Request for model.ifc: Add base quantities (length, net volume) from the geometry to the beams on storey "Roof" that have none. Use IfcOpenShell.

First a look at what the model holds.

```python
import ifcopenshell
import ifcopenshell.util.element
import ifcopenshell.util.unit

model = ifcopenshell.open("model.ifc")
print(model.schema)
for unit_type in ("LENGTHUNIT", "AREAUNIT", "VOLUMEUNIT"):
    print(unit_type, ifcopenshell.util.unit.calculate_unit_scale(model, unit_type))
storey = next(s for s in model.by_type("IfcBuildingStorey") if s.Name == "Roof")
beams = [e for e in ifcopenshell.util.element.get_decomposition(storey) if e.is_a("IfcBeam")]
for e in sorted(beams, key=lambda e: e.id()):
    print(e.id(), e.is_a(), e.Name, list(ifcopenshell.util.element.get_psets(e, qtos_only=True)), sep=" | ")
```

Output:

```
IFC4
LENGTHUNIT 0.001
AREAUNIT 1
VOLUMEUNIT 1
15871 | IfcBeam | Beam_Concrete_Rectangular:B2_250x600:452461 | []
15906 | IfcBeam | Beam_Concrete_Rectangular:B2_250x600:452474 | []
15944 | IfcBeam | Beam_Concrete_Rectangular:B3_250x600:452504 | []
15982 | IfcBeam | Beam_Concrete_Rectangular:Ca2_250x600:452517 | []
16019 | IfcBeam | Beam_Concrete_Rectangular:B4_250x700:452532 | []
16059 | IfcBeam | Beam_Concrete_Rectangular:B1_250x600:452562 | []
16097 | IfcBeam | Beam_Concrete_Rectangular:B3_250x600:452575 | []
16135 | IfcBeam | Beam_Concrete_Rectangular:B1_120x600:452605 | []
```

```python
import ifcopenshell
import ifcopenshell.api.pset
import ifcopenshell.geom
import ifcopenshell.util.element
import ifcopenshell.util.shape
import ifcopenshell.util.unit

model = ifcopenshell.open("model.ifc")
unit_scale = ifcopenshell.util.unit.calculate_unit_scale(model)
volume_scale = ifcopenshell.util.unit.calculate_unit_scale(model, "VOLUMEUNIT")
settings = ifcopenshell.geom.settings()

storey = next(s for s in model.by_type("IfcBuildingStorey") if s.Name == "Roof")
beams = [e for e in ifcopenshell.util.element.get_decomposition(storey) if e.is_a("IfcBeam")]

for e in sorted(beams, key=lambda e: e.id()):
    if ifcopenshell.util.element.get_psets(e, qtos_only=True, should_inherit=False):
        continue
    # Geometry comes back in metres, in the element's own axes.
    shape = ifcopenshell.geom.create_shape(settings, e)
    values = {
        "Length": ifcopenshell.util.shape.get_max_xyz(shape.geometry) / unit_scale,
        "NetVolume": ifcopenshell.util.shape.get_volume(shape.geometry) / volume_scale,
    }
    qto = ifcopenshell.api.pset.add_qto(model, product=e, name="Qto_BeamBaseQuantities")
    ifcopenshell.api.pset.edit_qto(model, qto=qto, properties=values)
    print(e.id(), {k: round(v, 3) for k, v in values.items()})

model.write("model-out.ifc")
```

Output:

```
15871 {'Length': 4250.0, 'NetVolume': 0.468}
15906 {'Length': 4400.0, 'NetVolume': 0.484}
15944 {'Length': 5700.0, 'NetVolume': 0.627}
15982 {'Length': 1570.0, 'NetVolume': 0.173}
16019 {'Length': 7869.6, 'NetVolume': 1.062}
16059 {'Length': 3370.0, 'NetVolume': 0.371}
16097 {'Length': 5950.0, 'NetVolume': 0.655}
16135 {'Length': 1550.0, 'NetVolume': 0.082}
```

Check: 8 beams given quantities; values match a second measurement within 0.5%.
